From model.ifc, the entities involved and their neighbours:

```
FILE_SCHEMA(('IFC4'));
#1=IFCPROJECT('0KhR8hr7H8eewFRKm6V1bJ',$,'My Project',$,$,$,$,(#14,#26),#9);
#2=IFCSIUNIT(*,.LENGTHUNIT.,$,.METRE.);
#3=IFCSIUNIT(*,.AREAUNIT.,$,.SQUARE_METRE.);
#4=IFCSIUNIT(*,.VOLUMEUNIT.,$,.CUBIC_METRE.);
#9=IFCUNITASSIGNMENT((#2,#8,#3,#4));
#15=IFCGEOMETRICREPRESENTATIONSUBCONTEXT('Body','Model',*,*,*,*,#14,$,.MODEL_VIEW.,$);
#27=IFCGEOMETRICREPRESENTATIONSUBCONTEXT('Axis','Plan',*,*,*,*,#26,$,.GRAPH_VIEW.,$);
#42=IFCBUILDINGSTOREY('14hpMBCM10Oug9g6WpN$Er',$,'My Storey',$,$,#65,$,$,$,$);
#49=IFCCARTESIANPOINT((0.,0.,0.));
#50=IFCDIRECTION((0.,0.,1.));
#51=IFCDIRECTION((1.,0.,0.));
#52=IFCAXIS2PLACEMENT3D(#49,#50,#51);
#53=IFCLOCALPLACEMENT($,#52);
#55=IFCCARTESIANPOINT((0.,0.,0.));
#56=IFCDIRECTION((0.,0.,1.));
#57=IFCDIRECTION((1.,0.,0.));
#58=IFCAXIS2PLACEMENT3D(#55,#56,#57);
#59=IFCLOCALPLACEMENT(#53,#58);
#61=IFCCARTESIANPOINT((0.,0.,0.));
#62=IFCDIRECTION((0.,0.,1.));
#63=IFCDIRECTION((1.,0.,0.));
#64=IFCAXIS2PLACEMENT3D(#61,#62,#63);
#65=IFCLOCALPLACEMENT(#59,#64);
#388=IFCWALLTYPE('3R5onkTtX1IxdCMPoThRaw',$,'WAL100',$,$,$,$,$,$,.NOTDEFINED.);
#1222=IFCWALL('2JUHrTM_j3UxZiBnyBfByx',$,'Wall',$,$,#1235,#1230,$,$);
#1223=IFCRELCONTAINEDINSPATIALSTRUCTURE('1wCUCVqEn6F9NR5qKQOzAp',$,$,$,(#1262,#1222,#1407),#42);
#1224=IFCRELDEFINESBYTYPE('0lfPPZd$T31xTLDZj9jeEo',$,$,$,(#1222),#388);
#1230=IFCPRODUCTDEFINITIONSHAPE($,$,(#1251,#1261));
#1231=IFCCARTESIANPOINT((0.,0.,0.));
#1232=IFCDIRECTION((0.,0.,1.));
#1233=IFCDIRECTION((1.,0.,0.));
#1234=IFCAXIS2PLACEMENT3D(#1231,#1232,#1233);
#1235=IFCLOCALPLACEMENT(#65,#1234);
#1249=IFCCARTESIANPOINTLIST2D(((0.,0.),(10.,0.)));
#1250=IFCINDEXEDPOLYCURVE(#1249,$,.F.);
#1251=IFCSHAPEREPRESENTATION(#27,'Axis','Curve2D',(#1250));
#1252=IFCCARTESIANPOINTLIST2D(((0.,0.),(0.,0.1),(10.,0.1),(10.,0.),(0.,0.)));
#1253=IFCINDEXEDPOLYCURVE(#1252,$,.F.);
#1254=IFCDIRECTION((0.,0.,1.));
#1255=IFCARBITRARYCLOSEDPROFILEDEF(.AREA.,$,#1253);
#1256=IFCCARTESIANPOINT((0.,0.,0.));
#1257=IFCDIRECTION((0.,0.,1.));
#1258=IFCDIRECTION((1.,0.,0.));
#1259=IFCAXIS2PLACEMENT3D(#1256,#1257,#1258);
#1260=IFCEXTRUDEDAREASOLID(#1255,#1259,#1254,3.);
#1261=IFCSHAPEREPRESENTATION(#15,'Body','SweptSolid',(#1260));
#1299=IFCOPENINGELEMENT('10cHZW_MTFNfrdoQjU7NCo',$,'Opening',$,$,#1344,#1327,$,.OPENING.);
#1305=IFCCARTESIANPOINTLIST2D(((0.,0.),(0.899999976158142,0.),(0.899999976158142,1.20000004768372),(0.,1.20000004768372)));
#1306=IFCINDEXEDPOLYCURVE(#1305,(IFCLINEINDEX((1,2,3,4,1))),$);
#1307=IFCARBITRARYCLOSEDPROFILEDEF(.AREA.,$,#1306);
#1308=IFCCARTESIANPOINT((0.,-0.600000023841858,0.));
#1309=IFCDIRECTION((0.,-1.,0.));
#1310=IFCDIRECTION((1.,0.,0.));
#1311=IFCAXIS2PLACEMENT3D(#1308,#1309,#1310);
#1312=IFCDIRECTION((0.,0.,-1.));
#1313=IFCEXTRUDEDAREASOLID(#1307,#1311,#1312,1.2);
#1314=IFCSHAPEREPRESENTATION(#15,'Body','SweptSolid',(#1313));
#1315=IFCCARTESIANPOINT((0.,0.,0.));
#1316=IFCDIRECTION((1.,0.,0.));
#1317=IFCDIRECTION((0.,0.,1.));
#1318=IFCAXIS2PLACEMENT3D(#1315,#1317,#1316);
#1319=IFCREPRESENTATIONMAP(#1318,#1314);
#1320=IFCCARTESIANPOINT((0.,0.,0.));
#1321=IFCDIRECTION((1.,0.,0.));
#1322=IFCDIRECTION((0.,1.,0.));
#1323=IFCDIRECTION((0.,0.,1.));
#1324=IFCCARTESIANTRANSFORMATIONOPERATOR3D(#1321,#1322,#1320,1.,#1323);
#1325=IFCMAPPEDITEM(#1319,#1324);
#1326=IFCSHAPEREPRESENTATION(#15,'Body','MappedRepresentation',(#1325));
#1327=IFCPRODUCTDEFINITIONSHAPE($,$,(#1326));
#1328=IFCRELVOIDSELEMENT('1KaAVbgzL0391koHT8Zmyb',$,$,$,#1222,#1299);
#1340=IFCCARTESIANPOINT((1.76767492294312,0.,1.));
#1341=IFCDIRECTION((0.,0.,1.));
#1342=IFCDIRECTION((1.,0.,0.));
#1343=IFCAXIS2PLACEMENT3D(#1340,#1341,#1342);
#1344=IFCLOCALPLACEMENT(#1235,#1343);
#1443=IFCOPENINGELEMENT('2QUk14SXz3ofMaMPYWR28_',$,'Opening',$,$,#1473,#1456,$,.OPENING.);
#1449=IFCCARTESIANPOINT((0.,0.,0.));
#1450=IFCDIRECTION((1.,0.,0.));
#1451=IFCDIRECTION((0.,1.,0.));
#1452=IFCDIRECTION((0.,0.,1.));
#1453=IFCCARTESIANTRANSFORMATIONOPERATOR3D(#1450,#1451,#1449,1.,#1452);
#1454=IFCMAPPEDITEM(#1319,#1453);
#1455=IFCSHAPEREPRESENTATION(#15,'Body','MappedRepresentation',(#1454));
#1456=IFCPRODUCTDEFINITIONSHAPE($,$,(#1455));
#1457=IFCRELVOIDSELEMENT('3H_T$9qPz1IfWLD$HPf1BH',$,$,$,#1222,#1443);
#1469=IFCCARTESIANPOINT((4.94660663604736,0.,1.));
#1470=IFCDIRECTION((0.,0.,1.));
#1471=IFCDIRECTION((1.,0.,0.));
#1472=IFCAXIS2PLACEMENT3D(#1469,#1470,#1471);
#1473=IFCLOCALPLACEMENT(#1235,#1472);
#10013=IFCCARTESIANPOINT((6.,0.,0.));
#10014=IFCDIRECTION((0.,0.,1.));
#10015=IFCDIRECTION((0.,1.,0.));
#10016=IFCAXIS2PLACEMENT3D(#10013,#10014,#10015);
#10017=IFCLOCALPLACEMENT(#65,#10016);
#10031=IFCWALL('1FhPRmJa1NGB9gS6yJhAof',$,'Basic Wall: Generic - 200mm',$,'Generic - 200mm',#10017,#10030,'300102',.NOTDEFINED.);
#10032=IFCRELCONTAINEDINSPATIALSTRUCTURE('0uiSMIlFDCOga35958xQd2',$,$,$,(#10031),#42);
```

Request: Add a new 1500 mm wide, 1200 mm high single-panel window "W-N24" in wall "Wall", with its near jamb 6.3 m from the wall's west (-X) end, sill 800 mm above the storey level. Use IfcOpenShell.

```python
import numpy as np
import ifcopenshell
import ifcopenshell.api.feature
import ifcopenshell.api.geometry
import ifcopenshell.api.root
import ifcopenshell.api.spatial
import ifcopenshell.geom
import ifcopenshell.util.element
import ifcopenshell.util.placement
import ifcopenshell.util.representation
import ifcopenshell.util.shape
import ifcopenshell.util.unit

model = ifcopenshell.open("model.ifc")
unit_scale = ifcopenshell.util.unit.calculate_unit_scale(model)
settings = ifcopenshell.geom.settings()


def volume(element):
    """Net volume in cubic metres, openings subtracted."""
    shape = ifcopenshell.geom.create_shape(settings, element)
    return ifcopenshell.util.shape.get_volume(shape.geometry)


wall = model.by_id(1222)
storey = ifcopenshell.util.element.get_container(wall, ifc_class="IfcBuildingStorey")
context = ifcopenshell.util.representation.get_context(model, "Model", "Body", "MODEL_VIEW")
before = volume(wall)

width, height, from_end, sill = 1.5, 1.2, 6.3, 0.8  # metres

# The wall runs along its own X axis, and the end named is its -X end.
wall_shape = ifcopenshell.geom.create_shape(settings, wall)
x, y, z = ifcopenshell.util.shape.get_vertices(wall_shape.geometry).T
start = x.min() + from_end
face, thickness = float(y.min()), float(y.max() - y.min())
wall_matrix = ifcopenshell.util.placement.get_local_placement(wall.ObjectPlacement)
level = ifcopenshell.util.placement.get_local_placement(storey.ObjectPlacement)[2, 3]


def in_wall(x, y):
    """Placement at x, y metres in the wall's axes, at sill height."""
    matrix = wall_matrix.copy()
    matrix[:, 3] = wall_matrix @ np.array([x / unit_scale, y / unit_scale, 0.0, 1.0])
    matrix[2, 3] = level + sill / unit_scale
    return matrix


# Opening: a box that overshoots both wall faces by 50 mm.
opening = ifcopenshell.api.root.create_entity(model, ifc_class="IfcOpeningElement", predefined_type="OPENING")
box = ifcopenshell.api.geometry.add_wall_representation(
    model, context=context, length=width, height=height, thickness=thickness + 0.1
)
ifcopenshell.api.geometry.assign_representation(model, product=opening, representation=box)
ifcopenshell.api.geometry.edit_object_placement(model, product=opening, matrix=in_wall(start, face - 0.05), is_si=False)
ifcopenshell.api.feature.add_feature(model, feature=opening, element=wall)

window = ifcopenshell.api.root.create_entity(model, ifc_class="IfcWindow", name="W-N24", predefined_type="WINDOW")
window.OverallWidth, window.OverallHeight = width / unit_scale, height / unit_scale
window.PartitioningType = "SINGLE_PANEL"
body = ifcopenshell.api.geometry.add_window_representation(
    model,
    context=context,
    overall_width=window.OverallWidth,
    overall_height=window.OverallHeight,
    partition_type="SINGLE_PANEL",
)
ifcopenshell.api.geometry.assign_representation(model, product=window, representation=body)
ifcopenshell.api.spatial.assign_container(model, products=[window], relating_structure=storey)
ifcopenshell.api.feature.add_filling(model, opening=opening, element=window)

# Centre the window in the wall's thickness.
ifcopenshell.api.geometry.edit_object_placement(model, product=window, matrix=in_wall(start, face), is_si=False)
window_shape = ifcopenshell.geom.create_shape(settings, window)
depth = ifcopenshell.util.shape.get_vertices(window_shape.geometry)[:, 1]
offset = face + thickness / 2 - (depth.min() + depth.max()) / 2
ifcopenshell.api.geometry.edit_object_placement(model, product=window, matrix=in_wall(start, offset), is_si=False)

after = volume(wall)

print(f"wall volume {before:.3f} -> {after:.3f} m3")

model.write("model_rev.ifc")
```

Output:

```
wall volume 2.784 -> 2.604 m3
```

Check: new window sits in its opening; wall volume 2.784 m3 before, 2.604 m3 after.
